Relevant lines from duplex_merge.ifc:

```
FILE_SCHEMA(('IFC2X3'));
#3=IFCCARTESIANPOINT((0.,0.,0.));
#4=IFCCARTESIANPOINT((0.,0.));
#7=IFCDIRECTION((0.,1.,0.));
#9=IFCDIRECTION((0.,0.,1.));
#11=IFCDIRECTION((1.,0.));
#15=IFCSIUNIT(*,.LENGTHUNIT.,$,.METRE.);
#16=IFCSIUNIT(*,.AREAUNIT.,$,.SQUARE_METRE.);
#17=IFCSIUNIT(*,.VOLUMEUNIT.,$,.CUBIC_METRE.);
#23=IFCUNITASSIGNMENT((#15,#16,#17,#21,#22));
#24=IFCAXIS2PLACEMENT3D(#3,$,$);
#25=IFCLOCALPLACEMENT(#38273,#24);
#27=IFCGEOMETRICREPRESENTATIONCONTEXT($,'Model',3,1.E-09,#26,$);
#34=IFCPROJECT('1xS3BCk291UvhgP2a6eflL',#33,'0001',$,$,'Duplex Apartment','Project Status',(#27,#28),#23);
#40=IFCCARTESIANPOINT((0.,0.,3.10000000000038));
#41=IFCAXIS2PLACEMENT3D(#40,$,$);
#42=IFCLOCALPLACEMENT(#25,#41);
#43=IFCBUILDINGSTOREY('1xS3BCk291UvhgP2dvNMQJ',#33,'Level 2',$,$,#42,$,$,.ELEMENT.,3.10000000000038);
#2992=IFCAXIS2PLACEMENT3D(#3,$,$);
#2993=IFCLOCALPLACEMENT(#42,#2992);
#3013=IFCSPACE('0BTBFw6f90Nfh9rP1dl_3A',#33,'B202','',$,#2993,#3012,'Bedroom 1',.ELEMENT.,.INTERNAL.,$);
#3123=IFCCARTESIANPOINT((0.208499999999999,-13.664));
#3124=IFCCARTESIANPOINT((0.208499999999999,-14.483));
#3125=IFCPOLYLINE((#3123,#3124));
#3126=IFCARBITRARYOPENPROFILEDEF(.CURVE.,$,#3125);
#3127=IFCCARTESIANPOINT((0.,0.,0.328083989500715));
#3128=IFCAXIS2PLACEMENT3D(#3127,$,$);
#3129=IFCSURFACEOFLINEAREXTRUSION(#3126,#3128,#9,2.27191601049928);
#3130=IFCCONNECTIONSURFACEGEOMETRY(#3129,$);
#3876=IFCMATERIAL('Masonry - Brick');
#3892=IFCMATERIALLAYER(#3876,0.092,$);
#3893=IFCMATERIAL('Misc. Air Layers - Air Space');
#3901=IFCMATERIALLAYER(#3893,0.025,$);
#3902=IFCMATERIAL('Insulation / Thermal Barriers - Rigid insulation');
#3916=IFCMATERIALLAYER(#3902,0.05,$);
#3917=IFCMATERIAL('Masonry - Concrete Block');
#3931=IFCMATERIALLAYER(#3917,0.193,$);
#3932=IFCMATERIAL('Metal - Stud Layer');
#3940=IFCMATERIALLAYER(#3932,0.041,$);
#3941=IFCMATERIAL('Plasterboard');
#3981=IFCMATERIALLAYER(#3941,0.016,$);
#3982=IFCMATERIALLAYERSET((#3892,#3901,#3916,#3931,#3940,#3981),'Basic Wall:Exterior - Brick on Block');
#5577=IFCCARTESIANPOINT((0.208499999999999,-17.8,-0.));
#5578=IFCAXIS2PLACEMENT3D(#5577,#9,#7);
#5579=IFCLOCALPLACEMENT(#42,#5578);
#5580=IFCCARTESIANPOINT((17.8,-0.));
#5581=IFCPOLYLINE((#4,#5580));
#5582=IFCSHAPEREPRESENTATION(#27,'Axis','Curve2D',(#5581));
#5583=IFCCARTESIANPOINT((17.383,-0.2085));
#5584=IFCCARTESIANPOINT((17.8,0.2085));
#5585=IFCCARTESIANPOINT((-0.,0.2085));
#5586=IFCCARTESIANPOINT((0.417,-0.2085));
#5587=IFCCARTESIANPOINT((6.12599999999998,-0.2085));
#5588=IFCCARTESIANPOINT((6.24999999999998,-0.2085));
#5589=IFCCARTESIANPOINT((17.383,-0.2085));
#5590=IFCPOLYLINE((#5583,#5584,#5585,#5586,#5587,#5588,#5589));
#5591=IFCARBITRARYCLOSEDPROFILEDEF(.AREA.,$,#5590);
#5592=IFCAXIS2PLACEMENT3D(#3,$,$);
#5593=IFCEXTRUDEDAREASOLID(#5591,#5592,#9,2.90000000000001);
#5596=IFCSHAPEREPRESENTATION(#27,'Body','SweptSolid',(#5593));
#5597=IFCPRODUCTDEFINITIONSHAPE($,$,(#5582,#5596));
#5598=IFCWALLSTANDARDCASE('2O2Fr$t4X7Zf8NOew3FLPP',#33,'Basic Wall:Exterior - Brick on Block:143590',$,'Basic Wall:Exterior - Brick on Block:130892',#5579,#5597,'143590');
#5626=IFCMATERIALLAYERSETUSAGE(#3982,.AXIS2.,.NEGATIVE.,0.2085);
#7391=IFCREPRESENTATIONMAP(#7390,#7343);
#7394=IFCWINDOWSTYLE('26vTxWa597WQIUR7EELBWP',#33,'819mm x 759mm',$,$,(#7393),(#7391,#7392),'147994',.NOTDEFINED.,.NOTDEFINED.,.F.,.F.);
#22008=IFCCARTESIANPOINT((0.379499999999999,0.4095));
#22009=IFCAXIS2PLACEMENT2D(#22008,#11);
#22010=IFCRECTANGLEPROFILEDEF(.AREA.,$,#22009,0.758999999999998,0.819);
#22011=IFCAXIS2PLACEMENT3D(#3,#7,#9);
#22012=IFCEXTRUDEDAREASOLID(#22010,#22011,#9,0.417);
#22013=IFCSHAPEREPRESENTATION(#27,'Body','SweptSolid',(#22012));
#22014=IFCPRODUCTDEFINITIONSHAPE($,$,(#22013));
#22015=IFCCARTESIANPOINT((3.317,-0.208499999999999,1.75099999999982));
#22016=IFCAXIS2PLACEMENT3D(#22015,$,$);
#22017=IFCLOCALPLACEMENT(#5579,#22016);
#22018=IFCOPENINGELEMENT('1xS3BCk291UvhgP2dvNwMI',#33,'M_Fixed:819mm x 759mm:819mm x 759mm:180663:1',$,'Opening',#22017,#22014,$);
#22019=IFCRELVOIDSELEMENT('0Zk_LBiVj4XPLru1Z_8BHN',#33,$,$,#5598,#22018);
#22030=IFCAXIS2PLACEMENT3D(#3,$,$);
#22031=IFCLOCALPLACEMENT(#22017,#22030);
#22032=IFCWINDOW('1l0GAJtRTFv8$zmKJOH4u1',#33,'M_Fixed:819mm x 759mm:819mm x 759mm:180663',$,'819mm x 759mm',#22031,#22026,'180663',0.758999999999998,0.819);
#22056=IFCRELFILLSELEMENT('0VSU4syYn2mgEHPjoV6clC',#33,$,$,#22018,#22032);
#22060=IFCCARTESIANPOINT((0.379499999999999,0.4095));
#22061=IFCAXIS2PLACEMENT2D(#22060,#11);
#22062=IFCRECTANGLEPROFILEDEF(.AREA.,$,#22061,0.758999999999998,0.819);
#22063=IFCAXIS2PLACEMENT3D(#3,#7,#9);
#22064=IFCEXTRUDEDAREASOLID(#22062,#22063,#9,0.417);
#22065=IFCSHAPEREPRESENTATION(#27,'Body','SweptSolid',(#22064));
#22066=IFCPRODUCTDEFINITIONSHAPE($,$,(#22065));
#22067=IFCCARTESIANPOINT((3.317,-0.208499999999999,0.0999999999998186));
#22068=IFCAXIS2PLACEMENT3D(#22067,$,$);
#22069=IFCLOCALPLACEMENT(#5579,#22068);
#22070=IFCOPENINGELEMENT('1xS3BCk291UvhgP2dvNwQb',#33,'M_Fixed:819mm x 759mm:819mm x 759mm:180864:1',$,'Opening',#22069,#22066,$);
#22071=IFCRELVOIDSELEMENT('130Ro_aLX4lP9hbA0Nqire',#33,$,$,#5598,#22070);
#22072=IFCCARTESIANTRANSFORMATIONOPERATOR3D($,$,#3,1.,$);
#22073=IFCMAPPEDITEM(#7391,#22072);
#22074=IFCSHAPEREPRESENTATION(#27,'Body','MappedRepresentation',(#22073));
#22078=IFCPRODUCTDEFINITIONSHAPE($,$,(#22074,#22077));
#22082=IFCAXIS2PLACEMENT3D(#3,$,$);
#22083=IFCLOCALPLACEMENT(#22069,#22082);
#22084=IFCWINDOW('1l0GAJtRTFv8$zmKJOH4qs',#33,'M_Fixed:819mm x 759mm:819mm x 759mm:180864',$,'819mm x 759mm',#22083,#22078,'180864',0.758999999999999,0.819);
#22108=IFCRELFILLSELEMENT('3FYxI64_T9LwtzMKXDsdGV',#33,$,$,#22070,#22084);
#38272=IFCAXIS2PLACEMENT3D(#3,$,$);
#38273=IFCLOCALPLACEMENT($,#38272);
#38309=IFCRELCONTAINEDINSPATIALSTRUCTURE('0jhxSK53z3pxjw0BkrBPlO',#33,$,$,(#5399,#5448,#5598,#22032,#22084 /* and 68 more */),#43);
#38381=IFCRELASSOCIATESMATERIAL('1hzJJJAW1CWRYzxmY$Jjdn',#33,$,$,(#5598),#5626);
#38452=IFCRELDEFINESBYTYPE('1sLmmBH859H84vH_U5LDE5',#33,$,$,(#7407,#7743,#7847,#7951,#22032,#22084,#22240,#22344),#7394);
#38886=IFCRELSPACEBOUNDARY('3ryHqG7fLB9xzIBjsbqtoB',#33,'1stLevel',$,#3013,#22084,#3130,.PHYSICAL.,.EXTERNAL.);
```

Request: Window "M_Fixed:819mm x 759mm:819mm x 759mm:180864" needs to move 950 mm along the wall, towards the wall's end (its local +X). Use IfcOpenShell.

```python
import numpy as np
import ifcopenshell
import ifcopenshell.api.geometry
import ifcopenshell.util.placement

model = ifcopenshell.open("duplex_merge.ifc")

window = model.by_id(22084)
opening = window.FillsVoids[0].RelatingOpeningElement
wall = opening.VoidsElements[0].RelatingBuildingElement

wall_matrix = ifcopenshell.util.placement.get_local_placement(wall.ObjectPlacement)
shift = wall_matrix[:3, 0] * 0.95
before = ifcopenshell.util.placement.get_local_placement(window.ObjectPlacement)[:3, 3].copy()

# The window is placed relative to its opening, so it follows when the opening moves.
matrix = ifcopenshell.util.placement.get_local_placement(opening.ObjectPlacement)
matrix[:3, 3] += shift
ifcopenshell.api.geometry.edit_object_placement(
    model, product=opening, matrix=matrix, is_si=False, should_transform_children=True
)

# Space boundary surfaces are stored in each space's coordinates; move them too.
for rel in window.ProvidesBoundaries:
    if not rel.ConnectionGeometry:
        continue
    surface = rel.ConnectionGeometry.SurfaceOnRelatingElement
    space_matrix = ifcopenshell.util.placement.get_local_placement(rel.RelatingSpace.ObjectPlacement)
    point = np.array(surface.Position.Location.Coordinates) + space_matrix[:3, :3].T @ shift
    surface.Position = model.createIfcAxis2Placement3D(
        model.createIfcCartesianPoint(point.tolist()), surface.Position.Axis, surface.Position.RefDirection
    )

after = ifcopenshell.util.placement.get_local_placement(window.ObjectPlacement)[:3, 3]
print("window moved by", (after - before).round(3) + 0.0)

model.write("duplex_merge_rev.ifc")
```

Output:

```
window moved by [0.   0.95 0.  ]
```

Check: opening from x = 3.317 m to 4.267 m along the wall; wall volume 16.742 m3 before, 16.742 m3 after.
